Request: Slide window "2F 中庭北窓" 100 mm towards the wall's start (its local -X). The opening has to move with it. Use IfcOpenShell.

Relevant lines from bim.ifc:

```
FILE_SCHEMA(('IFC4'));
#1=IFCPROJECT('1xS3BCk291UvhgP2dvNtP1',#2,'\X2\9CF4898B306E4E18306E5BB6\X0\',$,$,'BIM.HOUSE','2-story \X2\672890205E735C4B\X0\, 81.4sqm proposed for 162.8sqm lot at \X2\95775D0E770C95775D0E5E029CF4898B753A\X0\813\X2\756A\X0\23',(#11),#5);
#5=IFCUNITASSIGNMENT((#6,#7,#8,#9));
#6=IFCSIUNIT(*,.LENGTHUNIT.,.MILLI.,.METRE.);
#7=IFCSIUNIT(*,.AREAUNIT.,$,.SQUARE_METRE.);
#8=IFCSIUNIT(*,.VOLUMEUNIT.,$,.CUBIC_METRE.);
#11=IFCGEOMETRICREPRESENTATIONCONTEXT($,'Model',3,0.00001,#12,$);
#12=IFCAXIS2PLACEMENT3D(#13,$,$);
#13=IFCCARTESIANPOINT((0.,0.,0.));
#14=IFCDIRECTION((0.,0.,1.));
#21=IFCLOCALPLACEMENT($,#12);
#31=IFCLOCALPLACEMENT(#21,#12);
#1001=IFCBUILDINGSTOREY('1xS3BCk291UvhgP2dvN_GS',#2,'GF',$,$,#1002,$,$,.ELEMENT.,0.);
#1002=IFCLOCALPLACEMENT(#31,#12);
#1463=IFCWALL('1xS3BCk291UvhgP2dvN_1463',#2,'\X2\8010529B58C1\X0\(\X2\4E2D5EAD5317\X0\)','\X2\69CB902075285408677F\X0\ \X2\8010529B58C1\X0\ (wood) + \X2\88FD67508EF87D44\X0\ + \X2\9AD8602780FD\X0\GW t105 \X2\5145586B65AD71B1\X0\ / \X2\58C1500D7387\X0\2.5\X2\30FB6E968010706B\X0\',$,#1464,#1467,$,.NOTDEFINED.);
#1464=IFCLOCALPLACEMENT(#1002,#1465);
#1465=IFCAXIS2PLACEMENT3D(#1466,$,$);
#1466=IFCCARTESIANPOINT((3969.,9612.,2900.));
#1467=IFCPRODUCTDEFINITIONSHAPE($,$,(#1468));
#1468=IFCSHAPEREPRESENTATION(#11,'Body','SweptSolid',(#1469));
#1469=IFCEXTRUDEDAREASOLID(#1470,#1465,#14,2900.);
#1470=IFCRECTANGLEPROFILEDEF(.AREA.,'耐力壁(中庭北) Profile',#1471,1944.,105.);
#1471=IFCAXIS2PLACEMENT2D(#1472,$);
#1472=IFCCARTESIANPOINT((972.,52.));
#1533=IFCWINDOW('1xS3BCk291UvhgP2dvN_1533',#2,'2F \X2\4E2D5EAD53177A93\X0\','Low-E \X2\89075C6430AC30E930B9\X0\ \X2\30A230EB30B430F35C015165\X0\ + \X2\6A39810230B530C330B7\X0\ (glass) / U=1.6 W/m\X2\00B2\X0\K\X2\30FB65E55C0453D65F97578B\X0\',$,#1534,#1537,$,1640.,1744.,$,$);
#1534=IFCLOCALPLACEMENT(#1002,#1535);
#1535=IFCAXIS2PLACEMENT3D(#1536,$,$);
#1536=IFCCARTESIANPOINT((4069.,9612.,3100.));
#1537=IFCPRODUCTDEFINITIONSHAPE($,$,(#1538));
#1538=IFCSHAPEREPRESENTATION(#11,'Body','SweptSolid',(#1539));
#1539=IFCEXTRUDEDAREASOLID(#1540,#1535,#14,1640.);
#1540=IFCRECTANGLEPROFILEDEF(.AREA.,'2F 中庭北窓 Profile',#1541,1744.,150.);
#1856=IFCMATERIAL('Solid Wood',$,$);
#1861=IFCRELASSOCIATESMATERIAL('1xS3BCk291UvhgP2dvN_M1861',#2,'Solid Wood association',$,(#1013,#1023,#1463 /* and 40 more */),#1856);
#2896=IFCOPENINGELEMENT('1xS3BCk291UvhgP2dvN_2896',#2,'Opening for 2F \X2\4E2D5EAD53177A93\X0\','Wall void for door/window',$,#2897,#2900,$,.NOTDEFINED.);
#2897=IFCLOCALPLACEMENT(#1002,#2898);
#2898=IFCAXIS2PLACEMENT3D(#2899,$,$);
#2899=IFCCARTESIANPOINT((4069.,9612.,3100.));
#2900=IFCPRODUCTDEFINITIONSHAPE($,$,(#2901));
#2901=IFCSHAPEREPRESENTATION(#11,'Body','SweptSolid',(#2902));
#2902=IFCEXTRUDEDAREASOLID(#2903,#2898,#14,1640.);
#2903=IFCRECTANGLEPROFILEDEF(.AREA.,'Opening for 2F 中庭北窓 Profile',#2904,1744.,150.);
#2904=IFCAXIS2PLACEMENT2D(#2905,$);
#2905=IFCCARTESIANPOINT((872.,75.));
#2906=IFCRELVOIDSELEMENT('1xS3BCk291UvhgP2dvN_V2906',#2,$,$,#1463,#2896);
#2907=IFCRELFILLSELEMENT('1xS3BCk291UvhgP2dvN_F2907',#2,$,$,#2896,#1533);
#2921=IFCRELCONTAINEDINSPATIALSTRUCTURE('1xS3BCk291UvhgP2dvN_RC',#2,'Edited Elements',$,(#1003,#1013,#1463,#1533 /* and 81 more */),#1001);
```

```python
import ifcopenshell
import ifcopenshell.api.geometry
import ifcopenshell.util.placement

model = ifcopenshell.open("bim.ifc")

window = model.by_guid("1xS3BCk291UvhgP2dvN_1533")
opening = window.FillsVoids[0].RelatingOpeningElement
wall = opening.VoidsElements[0].RelatingBuildingElement

wall_matrix = ifcopenshell.util.placement.get_local_placement(wall.ObjectPlacement)
shift = wall_matrix[:3, 0] * -100.0
before = ifcopenshell.util.placement.get_local_placement(window.ObjectPlacement)[:3, 3].copy()

# The window is not placed relative to its opening, so move both.
for product in (opening, window):
    matrix = ifcopenshell.util.placement.get_local_placement(product.ObjectPlacement)
    matrix[:3, 3] += shift
    ifcopenshell.api.geometry.edit_object_placement(model, product=product, matrix=matrix, is_si=False)

after = ifcopenshell.util.placement.get_local_placement(window.ObjectPlacement)[:3, 3]
print("window moved by", (after - before).round(3) + 0.0)

model.write("bim_v2.ifc")
```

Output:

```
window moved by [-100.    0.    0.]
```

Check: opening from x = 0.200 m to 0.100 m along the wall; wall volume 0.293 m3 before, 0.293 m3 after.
